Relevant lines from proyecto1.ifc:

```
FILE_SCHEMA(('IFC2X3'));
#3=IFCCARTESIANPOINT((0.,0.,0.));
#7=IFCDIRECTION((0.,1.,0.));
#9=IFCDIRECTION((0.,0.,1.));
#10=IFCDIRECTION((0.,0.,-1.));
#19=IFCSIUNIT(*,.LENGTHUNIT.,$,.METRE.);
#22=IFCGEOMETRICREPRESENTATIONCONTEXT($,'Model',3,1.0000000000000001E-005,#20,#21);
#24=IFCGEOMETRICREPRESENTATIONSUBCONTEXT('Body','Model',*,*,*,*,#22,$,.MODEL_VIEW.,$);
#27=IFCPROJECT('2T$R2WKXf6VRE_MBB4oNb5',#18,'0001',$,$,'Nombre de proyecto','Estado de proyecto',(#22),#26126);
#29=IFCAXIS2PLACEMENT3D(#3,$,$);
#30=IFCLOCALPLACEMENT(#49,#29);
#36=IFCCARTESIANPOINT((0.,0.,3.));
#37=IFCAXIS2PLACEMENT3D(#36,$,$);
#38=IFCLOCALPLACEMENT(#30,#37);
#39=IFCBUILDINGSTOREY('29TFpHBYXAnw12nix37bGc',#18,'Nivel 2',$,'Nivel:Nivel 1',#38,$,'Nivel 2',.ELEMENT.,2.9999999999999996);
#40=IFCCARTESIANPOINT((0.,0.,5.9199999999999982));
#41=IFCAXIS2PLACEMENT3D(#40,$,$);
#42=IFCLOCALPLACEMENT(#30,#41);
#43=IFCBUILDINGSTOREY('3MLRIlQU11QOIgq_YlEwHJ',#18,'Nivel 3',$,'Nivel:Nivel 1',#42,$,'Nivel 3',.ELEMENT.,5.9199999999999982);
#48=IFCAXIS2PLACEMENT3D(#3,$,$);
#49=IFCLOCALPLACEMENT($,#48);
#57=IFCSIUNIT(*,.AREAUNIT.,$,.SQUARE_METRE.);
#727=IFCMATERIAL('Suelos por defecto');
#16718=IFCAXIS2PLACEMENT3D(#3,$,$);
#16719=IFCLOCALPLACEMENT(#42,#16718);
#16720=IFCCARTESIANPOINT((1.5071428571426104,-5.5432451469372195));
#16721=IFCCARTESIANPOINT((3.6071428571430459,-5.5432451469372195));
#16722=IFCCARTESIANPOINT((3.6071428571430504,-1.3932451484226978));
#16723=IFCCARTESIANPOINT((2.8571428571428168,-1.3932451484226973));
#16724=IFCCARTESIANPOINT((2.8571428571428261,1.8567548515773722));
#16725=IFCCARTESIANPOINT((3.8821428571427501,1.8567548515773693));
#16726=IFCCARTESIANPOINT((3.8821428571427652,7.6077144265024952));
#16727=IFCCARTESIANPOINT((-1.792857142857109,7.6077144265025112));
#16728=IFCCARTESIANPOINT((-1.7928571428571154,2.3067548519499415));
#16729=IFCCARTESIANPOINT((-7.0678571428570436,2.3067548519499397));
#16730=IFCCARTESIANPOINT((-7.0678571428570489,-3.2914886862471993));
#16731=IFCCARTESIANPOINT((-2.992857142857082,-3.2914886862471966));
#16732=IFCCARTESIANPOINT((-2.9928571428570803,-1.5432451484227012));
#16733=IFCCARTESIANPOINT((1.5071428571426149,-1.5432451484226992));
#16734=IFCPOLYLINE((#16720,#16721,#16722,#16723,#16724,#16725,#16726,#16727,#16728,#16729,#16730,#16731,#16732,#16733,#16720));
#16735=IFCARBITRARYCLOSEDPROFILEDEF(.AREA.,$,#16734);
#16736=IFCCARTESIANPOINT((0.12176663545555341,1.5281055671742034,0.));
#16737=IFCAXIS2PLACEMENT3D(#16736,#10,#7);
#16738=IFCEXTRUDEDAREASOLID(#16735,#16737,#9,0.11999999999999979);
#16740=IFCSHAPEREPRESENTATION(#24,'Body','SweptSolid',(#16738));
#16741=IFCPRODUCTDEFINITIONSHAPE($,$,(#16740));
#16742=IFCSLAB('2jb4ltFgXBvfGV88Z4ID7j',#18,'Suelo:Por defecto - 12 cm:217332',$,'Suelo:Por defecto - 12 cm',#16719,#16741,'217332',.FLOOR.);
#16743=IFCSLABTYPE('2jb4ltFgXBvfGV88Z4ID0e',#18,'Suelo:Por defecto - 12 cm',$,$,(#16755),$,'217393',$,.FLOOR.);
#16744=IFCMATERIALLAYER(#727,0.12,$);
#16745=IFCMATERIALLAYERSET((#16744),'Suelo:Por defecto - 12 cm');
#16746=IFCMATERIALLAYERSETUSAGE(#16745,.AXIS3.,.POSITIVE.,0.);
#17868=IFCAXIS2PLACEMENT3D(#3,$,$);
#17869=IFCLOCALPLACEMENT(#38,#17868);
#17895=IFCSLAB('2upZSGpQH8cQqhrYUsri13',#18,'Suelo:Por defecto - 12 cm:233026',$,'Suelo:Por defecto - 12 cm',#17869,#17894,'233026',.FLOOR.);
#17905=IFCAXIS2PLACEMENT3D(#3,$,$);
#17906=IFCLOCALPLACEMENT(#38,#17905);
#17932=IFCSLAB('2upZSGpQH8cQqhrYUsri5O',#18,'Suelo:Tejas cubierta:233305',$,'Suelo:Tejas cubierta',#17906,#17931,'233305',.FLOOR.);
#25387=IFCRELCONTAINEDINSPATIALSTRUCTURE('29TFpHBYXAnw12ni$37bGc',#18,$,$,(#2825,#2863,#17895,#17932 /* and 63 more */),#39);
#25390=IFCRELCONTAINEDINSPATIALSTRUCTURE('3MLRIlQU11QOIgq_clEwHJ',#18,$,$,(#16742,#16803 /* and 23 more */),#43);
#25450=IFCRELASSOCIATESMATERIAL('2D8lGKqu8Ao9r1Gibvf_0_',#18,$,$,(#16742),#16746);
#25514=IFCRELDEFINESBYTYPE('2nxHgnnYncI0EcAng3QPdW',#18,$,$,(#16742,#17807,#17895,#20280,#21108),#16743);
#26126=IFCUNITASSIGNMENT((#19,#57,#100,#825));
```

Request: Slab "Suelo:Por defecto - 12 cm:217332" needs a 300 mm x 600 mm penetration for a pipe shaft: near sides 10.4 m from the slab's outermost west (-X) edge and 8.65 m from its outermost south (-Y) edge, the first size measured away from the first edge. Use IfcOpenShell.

```python
import numpy as np
import ifcopenshell
import ifcopenshell.api.feature
import ifcopenshell.api.geometry
import ifcopenshell.api.root
import ifcopenshell.geom
import ifcopenshell.util.placement
import ifcopenshell.util.representation
import ifcopenshell.util.shape
import ifcopenshell.util.unit

model = ifcopenshell.open("proyecto1.ifc")
unit_scale = ifcopenshell.util.unit.calculate_unit_scale(model)
settings = ifcopenshell.geom.settings()


def volume(element):
    """Net volume in cubic metres, openings subtracted."""
    shape = ifcopenshell.geom.create_shape(settings, element)
    return ifcopenshell.util.shape.get_volume(shape.geometry)


slab = model.by_id(16742)
before = volume(slab)

# Extent in the slab's own axes, in metres. The edges named are its -X and -Y sides.
slab_shape = ifcopenshell.geom.create_shape(settings, slab)
vertices = ifcopenshell.util.shape.get_vertices(slab_shape.geometry)
x_min, y_min, bottom = vertices.min(axis=0)
top = vertices[:, 2].max()

opening = ifcopenshell.api.root.create_entity(model, ifc_class="IfcOpeningElement", name="Pipe shaft opening")
context = ifcopenshell.util.representation.get_context(model, "Model", "Body", "MODEL_VIEW")
width, depth = 0.3, 0.6
outline = [(0.0, 0.0), (width, 0.0), (width, depth), (0.0, depth), (0.0, 0.0)]
# Overshoot both faces by 50 mm so the cut is clean.
shape = ifcopenshell.api.geometry.add_slab_representation(
    model, context=context, depth=top - bottom + 0.1, polyline=outline
)
ifcopenshell.api.geometry.assign_representation(model, product=opening, representation=shape)

matrix = ifcopenshell.util.placement.get_local_placement(slab.ObjectPlacement)
matrix[:, 3] = matrix @ np.append(np.array([x_min + 10.4, y_min + 8.65, bottom - 0.05]) / unit_scale, 1.0)
ifcopenshell.api.geometry.edit_object_placement(model, product=opening, matrix=matrix, is_si=False)
ifcopenshell.api.feature.add_feature(model, feature=opening, element=slab)

after = volume(slab)

print(f"slab volume {before:.3f} -> {after:.3f} m3")

model.write("proyecto1_updated.ifc")
```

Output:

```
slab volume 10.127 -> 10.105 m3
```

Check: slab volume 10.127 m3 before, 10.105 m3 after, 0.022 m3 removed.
